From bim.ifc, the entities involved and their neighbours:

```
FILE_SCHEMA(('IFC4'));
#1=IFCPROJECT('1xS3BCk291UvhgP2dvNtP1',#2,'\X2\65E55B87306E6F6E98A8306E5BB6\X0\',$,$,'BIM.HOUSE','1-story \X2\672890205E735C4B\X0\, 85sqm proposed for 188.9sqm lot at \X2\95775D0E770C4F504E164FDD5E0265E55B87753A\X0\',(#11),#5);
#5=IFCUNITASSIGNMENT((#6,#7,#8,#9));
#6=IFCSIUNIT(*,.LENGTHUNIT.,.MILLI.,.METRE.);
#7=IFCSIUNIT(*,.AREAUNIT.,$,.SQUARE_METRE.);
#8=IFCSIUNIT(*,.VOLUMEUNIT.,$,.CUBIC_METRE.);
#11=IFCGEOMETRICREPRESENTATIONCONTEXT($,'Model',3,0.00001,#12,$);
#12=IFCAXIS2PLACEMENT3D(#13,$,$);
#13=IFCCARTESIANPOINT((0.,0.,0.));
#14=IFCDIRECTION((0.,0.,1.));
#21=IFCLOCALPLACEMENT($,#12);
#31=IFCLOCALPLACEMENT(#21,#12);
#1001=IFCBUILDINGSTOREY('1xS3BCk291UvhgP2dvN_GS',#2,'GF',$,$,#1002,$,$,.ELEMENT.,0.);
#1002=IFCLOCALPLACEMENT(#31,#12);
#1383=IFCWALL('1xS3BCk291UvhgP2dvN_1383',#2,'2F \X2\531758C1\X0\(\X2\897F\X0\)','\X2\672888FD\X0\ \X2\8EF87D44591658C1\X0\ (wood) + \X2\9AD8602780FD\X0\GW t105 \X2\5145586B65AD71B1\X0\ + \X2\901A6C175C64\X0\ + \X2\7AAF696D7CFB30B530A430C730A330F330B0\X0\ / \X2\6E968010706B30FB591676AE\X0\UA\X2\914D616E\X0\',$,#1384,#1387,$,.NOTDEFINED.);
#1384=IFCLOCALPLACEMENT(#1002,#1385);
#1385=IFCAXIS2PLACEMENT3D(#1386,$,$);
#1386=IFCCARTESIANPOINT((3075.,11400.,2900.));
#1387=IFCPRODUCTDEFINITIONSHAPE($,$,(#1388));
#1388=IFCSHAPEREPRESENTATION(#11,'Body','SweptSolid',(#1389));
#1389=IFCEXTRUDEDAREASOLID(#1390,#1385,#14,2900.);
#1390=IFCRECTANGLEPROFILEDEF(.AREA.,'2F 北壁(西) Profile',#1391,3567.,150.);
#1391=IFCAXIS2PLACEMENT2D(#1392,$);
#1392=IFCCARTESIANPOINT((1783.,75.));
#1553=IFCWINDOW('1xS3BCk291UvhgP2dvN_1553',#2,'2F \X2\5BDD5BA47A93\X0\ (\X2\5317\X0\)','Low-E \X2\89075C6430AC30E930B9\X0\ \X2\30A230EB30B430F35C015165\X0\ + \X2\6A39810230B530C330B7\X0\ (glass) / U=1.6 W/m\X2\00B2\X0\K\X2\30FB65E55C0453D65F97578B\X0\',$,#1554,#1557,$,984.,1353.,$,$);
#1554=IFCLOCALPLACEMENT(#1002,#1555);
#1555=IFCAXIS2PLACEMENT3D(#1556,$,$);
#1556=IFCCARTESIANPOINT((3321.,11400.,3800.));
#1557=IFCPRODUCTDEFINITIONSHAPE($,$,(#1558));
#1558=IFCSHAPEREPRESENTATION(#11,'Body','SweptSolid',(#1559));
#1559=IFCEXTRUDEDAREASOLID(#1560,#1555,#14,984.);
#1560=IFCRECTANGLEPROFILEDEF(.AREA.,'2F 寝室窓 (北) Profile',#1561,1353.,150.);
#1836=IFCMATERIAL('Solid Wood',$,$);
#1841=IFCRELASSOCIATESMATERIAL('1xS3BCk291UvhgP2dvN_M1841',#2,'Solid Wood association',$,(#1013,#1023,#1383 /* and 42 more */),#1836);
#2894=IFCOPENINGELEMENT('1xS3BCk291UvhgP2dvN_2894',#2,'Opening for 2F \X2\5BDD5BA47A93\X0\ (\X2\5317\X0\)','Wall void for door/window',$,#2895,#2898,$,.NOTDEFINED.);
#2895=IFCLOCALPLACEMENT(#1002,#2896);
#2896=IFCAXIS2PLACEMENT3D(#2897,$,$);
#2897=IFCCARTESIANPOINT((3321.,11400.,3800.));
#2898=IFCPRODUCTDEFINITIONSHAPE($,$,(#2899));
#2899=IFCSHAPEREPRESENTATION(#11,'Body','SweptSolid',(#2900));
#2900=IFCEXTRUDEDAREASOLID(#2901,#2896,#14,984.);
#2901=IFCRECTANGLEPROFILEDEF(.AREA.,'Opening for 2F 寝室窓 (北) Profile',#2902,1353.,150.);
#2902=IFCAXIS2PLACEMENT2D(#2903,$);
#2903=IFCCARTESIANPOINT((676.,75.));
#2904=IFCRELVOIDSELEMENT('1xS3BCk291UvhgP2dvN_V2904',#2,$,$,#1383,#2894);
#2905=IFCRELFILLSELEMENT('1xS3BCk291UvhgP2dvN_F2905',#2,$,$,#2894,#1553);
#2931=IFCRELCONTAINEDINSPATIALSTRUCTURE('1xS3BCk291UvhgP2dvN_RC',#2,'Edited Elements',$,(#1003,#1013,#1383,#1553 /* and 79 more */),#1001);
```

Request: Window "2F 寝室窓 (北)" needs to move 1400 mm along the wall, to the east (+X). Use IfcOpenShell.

```python
import ifcopenshell
import ifcopenshell.api.geometry
import ifcopenshell.util.placement
import ifcopenshell.util.unit

model = ifcopenshell.open("bim.ifc")
unit_scale = ifcopenshell.util.unit.calculate_unit_scale(model)

window = model.by_guid("1xS3BCk291UvhgP2dvN_1553")
opening = window.FillsVoids[0].RelatingOpeningElement
wall = opening.VoidsElements[0].RelatingBuildingElement

wall_matrix = ifcopenshell.util.placement.get_local_placement(wall.ObjectPlacement)
shift = wall_matrix[:3, 0] * 1.4 / unit_scale
before = ifcopenshell.util.placement.get_local_placement(window.ObjectPlacement)[:3, 3].copy()

# The window is not placed relative to its opening, so move both.
for product in (opening, window):
    matrix = ifcopenshell.util.placement.get_local_placement(product.ObjectPlacement)
    matrix[:3, 3] += shift
    ifcopenshell.api.geometry.edit_object_placement(model, product=product, matrix=matrix, is_si=False)

after = ifcopenshell.util.placement.get_local_placement(window.ObjectPlacement)[:3, 3]
print("window moved by", (after - before).round(3) + 0.0)

model.write("bim_updated.ifc")
```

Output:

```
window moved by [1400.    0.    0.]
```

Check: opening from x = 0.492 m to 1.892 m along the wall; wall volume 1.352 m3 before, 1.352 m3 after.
